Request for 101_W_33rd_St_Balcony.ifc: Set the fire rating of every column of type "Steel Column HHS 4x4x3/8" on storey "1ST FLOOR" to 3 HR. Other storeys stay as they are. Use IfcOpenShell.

First a look at what the model holds.

```python
import ifcopenshell
import ifcopenshell.util.element

model = ifcopenshell.open("101_W_33rd_St_Balcony.ifc")
print(model.schema)
storey = next(s for s in model.by_type("IfcBuildingStorey") if s.Name == "1ST FLOOR")
columns = [e for e in ifcopenshell.util.element.get_decomposition(storey) if e.is_a("IfcColumn")]
seen = {}
for e in columns:
    element_type = ifcopenshell.util.element.get_type(e)
    key = (element_type.Name if element_type != e and element_type else None, ifcopenshell.util.element.get_pset(e, "Pset_ColumnCommon", "FireRating"))
    seen[key] = seen.get(key, 0) + 1
for (name, value), count in sorted(seen.items(), key=str):
    print(count, "x", name, "|", value)
```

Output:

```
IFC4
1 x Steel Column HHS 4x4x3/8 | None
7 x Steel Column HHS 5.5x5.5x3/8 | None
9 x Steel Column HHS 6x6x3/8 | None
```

```python
import ifcopenshell
import ifcopenshell.api.pset
import ifcopenshell.util.element

model = ifcopenshell.open("101_W_33rd_St_Balcony.ifc")

storey = next(s for s in model.by_type("IfcBuildingStorey") if s.Name == "1ST FLOOR")
columns = [e for e in ifcopenshell.util.element.get_decomposition(storey) if e.is_a("IfcColumn")]

count = 0
for e in columns:
    element_type = ifcopenshell.util.element.get_type(e)
    if element_type in (None, e) or element_type.Name != "Steel Column HHS 4x4x3/8":
        continue
    # add_pset returns the element's existing set when there is one.
    pset = ifcopenshell.api.pset.add_pset(model, product=e, name="Pset_ColumnCommon")
    ifcopenshell.api.pset.edit_pset(model, pset=pset, properties={"FireRating": "3 HR"})
    count += 1

print(count, "columns updated")

model.write("101_W_33rd_St_Balcony_edited.ifc")
```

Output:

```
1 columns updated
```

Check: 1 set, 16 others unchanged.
